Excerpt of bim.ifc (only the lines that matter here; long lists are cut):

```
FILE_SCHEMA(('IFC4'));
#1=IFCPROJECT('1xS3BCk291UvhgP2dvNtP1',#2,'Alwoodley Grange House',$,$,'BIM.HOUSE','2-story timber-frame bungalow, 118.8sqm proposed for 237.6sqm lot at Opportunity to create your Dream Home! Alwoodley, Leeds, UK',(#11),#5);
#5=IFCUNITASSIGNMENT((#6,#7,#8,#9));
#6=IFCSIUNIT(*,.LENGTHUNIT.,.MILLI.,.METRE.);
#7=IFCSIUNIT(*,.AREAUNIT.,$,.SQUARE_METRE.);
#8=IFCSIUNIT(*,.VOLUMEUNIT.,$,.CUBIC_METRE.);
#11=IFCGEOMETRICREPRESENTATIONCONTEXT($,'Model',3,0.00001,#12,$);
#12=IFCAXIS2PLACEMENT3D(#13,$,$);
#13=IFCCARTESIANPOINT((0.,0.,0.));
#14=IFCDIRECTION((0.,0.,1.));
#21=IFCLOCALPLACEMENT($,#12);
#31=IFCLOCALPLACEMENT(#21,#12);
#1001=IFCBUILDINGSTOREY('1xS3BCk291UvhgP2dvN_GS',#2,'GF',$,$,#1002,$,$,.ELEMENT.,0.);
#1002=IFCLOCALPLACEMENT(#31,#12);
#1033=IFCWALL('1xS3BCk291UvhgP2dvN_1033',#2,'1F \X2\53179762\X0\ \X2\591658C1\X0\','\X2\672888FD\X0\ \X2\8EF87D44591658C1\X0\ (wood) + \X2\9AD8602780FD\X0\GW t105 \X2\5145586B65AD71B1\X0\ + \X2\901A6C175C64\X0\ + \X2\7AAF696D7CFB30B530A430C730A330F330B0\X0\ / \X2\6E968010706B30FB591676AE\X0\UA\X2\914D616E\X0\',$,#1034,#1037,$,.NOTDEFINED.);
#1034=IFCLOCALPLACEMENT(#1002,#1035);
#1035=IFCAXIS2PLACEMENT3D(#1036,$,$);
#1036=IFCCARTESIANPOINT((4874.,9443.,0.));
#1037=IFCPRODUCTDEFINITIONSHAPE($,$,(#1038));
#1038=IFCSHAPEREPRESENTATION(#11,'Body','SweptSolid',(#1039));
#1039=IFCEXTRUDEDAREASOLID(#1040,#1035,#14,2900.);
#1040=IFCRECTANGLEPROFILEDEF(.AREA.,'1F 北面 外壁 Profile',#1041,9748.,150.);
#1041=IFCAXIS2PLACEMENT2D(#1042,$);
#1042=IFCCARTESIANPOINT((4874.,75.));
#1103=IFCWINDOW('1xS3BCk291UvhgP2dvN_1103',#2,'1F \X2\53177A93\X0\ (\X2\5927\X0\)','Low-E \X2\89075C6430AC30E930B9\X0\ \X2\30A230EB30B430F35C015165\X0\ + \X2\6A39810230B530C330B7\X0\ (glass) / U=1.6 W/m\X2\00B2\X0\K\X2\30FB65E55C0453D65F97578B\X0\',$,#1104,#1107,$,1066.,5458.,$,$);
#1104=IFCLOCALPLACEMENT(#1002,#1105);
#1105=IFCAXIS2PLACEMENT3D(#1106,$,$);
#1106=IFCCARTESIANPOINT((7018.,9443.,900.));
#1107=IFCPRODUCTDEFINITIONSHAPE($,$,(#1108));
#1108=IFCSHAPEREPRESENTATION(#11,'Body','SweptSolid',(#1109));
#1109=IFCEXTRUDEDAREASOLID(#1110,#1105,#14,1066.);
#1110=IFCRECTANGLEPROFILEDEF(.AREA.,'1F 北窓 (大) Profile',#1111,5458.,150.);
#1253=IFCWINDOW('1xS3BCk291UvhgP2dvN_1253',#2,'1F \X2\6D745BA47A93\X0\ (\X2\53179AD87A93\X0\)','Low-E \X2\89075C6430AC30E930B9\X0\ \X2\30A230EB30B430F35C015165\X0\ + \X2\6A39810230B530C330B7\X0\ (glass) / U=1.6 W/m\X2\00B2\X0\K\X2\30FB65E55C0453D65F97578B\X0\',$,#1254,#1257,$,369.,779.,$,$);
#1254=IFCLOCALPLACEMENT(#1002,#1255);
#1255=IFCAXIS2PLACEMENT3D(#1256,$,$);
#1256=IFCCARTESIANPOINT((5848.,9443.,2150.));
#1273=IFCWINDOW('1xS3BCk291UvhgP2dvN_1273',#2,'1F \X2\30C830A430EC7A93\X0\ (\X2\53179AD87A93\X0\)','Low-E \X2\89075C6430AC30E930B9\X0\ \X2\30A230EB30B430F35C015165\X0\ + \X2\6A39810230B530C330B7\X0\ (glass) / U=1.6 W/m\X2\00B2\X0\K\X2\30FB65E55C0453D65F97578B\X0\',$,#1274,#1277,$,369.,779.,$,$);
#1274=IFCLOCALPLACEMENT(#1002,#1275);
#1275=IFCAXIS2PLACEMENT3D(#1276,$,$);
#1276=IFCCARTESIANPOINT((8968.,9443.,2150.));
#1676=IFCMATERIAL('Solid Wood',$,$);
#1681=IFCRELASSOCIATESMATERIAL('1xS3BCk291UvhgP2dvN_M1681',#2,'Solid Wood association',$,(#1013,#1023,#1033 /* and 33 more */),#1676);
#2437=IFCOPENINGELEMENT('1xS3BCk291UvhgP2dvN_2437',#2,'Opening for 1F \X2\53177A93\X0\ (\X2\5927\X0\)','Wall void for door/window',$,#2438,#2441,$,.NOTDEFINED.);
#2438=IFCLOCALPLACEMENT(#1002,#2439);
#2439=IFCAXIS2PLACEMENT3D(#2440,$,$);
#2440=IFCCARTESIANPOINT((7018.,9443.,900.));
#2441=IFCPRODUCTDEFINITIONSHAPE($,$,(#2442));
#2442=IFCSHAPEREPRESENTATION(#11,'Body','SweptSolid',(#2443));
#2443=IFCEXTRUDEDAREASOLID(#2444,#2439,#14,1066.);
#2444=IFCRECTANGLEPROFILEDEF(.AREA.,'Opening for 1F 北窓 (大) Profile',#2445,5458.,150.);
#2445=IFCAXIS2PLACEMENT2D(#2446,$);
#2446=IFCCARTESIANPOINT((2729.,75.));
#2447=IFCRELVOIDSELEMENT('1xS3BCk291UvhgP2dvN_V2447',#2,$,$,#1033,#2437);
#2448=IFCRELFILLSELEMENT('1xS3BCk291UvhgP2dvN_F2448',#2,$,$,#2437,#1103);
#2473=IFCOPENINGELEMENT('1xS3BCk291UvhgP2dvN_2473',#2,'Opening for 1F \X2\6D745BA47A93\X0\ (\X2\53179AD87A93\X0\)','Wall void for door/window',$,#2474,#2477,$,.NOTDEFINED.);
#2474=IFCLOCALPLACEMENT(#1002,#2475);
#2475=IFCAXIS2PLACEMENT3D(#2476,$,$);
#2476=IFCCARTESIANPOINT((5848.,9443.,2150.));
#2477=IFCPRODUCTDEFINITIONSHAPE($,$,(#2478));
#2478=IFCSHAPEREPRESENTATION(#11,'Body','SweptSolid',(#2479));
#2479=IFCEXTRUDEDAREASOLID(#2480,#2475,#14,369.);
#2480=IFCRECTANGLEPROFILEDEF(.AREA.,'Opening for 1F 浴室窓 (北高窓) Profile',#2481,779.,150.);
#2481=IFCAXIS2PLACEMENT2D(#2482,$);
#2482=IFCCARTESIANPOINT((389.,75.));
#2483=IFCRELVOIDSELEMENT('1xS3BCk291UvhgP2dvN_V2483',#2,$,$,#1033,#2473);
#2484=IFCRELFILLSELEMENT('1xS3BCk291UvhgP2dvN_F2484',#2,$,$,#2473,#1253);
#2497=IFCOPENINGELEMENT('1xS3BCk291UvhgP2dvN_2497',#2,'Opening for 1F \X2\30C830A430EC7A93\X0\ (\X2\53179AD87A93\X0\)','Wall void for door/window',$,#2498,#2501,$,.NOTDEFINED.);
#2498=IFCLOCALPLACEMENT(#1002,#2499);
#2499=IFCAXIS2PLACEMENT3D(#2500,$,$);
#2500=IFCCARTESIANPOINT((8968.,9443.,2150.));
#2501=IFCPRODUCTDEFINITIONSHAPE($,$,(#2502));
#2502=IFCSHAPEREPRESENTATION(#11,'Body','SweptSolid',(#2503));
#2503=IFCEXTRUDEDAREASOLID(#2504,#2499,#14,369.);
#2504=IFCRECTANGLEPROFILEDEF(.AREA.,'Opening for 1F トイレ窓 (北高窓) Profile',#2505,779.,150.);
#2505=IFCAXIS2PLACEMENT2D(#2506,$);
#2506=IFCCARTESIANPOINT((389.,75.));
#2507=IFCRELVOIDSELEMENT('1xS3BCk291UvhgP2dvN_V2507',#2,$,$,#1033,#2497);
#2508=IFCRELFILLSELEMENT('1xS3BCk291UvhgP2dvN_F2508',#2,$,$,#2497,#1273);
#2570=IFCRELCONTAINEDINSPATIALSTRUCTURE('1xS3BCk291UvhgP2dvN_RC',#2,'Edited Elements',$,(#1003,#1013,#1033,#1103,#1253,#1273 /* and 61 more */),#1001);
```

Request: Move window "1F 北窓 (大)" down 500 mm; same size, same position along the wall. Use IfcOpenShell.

```python
import numpy as np
import ifcopenshell
import ifcopenshell.api.geometry
import ifcopenshell.util.placement
import ifcopenshell.util.unit

model = ifcopenshell.open("bim.ifc")
unit_scale = ifcopenshell.util.unit.calculate_unit_scale(model)

window = model.by_guid("1xS3BCk291UvhgP2dvN_1103")
opening = window.FillsVoids[0].RelatingOpeningElement
dz = -0.5 / unit_scale

shift = np.array([0.0, 0.0, dz])
# The window is not placed relative to its opening, so move both.
for product in (opening, window):
    matrix = ifcopenshell.util.placement.get_local_placement(product.ObjectPlacement)
    matrix[:3, 3] += shift
    ifcopenshell.api.geometry.edit_object_placement(model, product=product, matrix=matrix, is_si=False)

print(f"moved by {dz * unit_scale:+.3f} m")

model.write("bim_v2.ifc")
```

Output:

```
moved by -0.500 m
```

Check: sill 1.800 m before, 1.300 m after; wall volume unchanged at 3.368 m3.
